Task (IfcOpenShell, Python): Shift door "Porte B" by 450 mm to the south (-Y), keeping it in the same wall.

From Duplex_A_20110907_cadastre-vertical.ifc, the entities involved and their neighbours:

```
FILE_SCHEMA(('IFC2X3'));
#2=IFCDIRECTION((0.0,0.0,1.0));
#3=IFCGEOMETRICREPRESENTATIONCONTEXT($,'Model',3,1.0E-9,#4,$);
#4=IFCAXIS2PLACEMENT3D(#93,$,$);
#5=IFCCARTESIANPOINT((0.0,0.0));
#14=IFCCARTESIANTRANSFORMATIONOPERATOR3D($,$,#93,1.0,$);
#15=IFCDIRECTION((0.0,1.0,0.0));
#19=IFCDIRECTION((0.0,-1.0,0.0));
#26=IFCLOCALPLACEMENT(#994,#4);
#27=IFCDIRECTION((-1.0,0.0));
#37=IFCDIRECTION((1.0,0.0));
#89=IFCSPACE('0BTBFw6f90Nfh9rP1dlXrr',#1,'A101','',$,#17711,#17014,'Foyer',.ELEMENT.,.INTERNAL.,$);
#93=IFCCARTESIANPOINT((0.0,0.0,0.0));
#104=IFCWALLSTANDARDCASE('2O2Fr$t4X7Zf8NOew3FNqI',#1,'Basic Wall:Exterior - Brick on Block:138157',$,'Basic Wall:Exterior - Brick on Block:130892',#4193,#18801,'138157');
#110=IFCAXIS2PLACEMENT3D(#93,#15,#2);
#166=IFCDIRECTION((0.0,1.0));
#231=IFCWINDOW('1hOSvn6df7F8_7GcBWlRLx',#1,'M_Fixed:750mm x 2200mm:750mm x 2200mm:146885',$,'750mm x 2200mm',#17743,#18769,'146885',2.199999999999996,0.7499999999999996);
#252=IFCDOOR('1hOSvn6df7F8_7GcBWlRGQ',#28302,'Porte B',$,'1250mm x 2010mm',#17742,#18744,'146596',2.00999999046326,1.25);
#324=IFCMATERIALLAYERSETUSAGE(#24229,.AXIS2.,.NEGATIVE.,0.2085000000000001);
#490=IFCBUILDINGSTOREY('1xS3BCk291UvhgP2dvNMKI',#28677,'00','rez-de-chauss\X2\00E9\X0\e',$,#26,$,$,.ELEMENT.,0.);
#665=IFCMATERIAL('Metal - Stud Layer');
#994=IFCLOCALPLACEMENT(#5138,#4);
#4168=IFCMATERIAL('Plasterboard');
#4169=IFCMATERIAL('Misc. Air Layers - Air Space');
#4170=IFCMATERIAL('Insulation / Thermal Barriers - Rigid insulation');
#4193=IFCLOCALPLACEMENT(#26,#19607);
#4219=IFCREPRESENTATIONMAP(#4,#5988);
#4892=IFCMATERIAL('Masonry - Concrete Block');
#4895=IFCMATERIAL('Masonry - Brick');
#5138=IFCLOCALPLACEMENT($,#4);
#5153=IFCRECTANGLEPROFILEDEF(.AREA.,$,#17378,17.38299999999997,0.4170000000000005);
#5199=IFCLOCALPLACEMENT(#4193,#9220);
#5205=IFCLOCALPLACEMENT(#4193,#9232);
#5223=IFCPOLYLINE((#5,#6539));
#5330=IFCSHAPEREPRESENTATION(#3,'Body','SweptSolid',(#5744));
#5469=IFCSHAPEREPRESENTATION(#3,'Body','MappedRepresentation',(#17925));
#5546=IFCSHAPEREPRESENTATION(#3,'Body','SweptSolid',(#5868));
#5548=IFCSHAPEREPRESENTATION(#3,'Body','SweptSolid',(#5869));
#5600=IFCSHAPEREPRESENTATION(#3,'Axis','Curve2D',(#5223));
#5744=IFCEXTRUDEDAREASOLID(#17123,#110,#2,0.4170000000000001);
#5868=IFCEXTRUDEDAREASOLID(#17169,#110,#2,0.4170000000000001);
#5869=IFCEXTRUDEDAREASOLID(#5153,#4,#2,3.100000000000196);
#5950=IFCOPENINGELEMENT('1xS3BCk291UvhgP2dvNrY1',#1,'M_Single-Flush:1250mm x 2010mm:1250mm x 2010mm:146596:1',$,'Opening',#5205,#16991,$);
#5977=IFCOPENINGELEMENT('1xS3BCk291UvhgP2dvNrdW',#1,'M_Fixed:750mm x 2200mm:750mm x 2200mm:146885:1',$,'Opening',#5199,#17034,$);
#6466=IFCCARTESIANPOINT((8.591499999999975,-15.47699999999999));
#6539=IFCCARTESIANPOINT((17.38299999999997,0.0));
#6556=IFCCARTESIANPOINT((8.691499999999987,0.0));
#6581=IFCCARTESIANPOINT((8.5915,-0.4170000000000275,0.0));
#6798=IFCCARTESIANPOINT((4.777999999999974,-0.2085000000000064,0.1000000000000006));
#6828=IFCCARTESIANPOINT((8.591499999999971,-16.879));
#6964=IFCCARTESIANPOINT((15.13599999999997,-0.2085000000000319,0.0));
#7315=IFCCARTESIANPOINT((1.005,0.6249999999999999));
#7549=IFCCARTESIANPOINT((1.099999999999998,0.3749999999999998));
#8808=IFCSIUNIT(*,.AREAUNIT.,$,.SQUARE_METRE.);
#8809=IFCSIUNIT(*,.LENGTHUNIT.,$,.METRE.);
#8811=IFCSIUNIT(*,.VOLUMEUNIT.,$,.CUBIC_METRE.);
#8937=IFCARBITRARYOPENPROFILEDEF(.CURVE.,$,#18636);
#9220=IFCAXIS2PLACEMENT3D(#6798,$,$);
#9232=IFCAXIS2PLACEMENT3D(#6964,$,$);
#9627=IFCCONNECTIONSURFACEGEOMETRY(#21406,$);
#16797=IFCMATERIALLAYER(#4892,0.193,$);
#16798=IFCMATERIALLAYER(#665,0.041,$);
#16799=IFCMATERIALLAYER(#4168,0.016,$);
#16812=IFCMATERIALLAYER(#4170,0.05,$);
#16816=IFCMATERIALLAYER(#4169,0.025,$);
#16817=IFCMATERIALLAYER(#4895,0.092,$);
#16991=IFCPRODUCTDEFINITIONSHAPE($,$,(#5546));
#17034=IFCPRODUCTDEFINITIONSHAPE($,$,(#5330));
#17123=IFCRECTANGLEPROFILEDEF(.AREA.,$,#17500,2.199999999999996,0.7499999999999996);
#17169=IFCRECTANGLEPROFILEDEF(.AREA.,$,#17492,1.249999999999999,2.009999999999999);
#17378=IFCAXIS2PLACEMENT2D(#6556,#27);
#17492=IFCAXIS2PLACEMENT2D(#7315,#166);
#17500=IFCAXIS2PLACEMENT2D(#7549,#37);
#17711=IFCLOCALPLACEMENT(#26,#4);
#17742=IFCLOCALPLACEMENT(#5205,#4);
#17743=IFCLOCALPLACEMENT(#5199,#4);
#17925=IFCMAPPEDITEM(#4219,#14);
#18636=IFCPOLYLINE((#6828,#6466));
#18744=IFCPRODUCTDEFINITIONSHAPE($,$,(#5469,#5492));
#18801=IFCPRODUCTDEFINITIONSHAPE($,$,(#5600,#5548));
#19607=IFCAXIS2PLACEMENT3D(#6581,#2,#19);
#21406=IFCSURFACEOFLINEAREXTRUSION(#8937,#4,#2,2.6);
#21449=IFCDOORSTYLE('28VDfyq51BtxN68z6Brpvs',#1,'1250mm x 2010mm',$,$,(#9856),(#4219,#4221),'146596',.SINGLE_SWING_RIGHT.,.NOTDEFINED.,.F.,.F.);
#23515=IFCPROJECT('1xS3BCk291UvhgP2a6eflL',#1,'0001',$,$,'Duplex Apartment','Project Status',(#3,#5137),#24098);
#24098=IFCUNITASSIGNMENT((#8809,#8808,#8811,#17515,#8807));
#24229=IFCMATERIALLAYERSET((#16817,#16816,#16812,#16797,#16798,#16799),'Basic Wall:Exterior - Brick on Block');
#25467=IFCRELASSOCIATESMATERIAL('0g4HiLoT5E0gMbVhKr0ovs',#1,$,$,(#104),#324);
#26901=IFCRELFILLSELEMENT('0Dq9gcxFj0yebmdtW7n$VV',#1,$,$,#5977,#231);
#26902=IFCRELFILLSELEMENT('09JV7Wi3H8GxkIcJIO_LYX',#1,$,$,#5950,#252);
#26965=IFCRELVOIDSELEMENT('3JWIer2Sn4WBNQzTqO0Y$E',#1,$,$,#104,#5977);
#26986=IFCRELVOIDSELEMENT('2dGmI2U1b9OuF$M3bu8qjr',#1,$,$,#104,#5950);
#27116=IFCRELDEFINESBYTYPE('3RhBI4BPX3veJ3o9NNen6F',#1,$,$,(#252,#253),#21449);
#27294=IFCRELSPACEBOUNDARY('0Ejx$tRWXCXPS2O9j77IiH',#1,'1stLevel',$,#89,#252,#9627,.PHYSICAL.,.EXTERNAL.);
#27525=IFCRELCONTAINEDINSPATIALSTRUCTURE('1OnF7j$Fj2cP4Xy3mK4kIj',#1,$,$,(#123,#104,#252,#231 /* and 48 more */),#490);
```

```python
import numpy as np
import ifcopenshell
import ifcopenshell.api.geometry
import ifcopenshell.util.placement
import ifcopenshell.util.unit

model = ifcopenshell.open("Duplex_A_20110907_cadastre-vertical.ifc")
unit_scale = ifcopenshell.util.unit.calculate_unit_scale(model)

door = model.by_guid("1hOSvn6df7F8_7GcBWlRGQ")
opening = door.FillsVoids[0].RelatingOpeningElement
wall = opening.VoidsElements[0].RelatingBuildingElement

wall_matrix = ifcopenshell.util.placement.get_local_placement(wall.ObjectPlacement)
shift = wall_matrix[:3, 0] * 0.45 / unit_scale
before = ifcopenshell.util.placement.get_local_placement(door.ObjectPlacement)[:3, 3].copy()

# The door is placed relative to its opening, so it follows when the opening moves.
matrix = ifcopenshell.util.placement.get_local_placement(opening.ObjectPlacement)
matrix[:3, 3] += shift
ifcopenshell.api.geometry.edit_object_placement(
    model, product=opening, matrix=matrix, is_si=False, should_transform_children=True
)

# Space boundary surfaces are stored in each space's coordinates; move them too.
for rel in door.ProvidesBoundaries:
    if not rel.ConnectionGeometry:
        continue
    surface = rel.ConnectionGeometry.SurfaceOnRelatingElement
    space_matrix = ifcopenshell.util.placement.get_local_placement(rel.RelatingSpace.ObjectPlacement)
    point = np.array(surface.Position.Location.Coordinates) + space_matrix[:3, :3].T @ shift
    surface.Position = model.createIfcAxis2Placement3D(
        model.createIfcCartesianPoint(point.tolist()), surface.Position.Axis, surface.Position.RefDirection
    )

after = ifcopenshell.util.placement.get_local_placement(door.ObjectPlacement)[:3, 3]
print("door moved by", (after - before).round(3) + 0.0)

model.write("Duplex_A_20110907_cadastre-vertical_v2.ifc")
```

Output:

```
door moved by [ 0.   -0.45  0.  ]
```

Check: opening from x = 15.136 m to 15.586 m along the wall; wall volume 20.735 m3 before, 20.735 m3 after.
